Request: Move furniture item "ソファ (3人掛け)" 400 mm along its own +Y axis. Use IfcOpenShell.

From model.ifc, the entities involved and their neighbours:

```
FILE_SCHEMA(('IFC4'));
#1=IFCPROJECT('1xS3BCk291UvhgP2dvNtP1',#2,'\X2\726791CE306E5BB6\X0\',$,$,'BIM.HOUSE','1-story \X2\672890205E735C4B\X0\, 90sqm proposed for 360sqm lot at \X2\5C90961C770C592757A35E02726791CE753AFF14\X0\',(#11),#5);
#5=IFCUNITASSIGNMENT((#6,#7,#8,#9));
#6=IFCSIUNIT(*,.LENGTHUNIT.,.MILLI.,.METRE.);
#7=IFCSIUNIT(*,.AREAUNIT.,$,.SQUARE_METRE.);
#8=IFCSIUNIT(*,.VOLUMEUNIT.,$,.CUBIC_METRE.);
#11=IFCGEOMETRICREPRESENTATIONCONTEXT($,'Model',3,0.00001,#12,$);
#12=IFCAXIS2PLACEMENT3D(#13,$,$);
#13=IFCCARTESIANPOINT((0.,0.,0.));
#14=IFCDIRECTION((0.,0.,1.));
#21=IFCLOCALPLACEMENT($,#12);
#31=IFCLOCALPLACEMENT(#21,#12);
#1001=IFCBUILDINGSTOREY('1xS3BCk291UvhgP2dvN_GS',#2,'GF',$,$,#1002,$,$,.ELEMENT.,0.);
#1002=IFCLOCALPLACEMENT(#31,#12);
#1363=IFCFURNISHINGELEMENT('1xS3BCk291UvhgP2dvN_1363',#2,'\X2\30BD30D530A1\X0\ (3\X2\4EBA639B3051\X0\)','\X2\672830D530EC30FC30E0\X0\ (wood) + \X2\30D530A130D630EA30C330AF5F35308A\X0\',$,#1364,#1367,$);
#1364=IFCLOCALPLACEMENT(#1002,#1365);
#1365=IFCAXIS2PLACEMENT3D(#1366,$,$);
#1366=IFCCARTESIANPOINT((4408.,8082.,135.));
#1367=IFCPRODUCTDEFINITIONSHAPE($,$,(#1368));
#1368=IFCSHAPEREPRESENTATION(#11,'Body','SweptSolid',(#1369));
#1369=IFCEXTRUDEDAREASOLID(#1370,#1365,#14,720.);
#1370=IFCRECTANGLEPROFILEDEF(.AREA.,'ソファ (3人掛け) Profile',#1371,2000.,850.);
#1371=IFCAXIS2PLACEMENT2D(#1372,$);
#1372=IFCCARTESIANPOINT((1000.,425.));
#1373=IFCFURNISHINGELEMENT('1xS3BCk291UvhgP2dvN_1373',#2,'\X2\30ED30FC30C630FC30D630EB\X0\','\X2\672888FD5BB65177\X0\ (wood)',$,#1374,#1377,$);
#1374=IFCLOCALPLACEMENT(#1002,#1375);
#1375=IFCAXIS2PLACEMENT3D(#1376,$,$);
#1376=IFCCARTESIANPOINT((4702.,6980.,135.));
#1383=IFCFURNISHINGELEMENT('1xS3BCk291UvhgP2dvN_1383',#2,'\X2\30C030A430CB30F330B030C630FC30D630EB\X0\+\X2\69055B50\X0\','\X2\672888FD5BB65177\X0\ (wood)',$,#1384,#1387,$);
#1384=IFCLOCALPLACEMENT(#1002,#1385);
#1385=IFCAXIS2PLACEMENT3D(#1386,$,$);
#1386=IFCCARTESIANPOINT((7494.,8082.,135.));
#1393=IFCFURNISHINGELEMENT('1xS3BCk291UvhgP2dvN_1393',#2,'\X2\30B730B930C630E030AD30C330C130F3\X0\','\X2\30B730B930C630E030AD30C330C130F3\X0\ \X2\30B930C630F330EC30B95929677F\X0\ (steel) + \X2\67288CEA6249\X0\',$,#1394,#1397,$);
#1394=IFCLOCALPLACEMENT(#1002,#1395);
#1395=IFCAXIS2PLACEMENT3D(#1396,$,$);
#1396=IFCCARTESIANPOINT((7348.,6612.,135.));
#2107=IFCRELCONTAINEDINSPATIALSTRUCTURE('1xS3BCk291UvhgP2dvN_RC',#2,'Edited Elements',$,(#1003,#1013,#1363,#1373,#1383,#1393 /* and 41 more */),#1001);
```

```python
import ifcopenshell
import ifcopenshell.api.geometry
import ifcopenshell.util.placement
import ifcopenshell.util.unit

model = ifcopenshell.open("model.ifc")
unit_scale = ifcopenshell.util.unit.calculate_unit_scale(model)

item = model.by_guid("1xS3BCk291UvhgP2dvN_1363")
matrix = ifcopenshell.util.placement.get_local_placement(item.ObjectPlacement)
matrix[:3, 3] += matrix[:3, 1] * 0.4 / unit_scale
ifcopenshell.api.geometry.edit_object_placement(model, product=item, matrix=matrix, is_si=False)

print(ifcopenshell.util.placement.get_local_placement(item.ObjectPlacement).round(3) + 0.0)

model.write("model_edited.ifc")
```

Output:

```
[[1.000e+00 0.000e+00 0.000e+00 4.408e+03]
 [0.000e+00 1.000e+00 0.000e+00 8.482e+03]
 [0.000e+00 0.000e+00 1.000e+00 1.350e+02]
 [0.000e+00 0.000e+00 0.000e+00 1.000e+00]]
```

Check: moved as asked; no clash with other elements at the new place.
